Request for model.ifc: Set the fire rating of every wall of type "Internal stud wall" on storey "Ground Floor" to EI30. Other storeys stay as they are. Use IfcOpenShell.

First a look at what the model holds.

```python
import ifcopenshell
import ifcopenshell.util.element

model = ifcopenshell.open("model.ifc")
print(model.schema)
storey = next(s for s in model.by_type("IfcBuildingStorey") if s.Name == "Ground Floor")
walls = [e for e in ifcopenshell.util.element.get_decomposition(storey) if e.is_a("IfcWall")]
seen = {}
for e in walls:
    element_type = ifcopenshell.util.element.get_type(e)
    key = (element_type.Name if element_type != e and element_type else None, ifcopenshell.util.element.get_pset(e, "Pset_WallCommon", "FireRating"))
    seen[key] = seen.get(key, 0) + 1
for (name, value), count in sorted(seen.items(), key=str):
    print(count, "x", name, "|", value)
```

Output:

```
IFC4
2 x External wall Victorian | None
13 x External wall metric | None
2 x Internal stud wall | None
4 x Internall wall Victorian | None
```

```python
import ifcopenshell
import ifcopenshell.api.pset
import ifcopenshell.util.element

model = ifcopenshell.open("model.ifc")

storey = next(s for s in model.by_type("IfcBuildingStorey") if s.Name == "Ground Floor")
walls = [e for e in ifcopenshell.util.element.get_decomposition(storey) if e.is_a("IfcWall")]

count = 0
for e in walls:
    element_type = ifcopenshell.util.element.get_type(e)
    if element_type in (None, e) or element_type.Name != "Internal stud wall":
        continue
    # add_pset returns the element's existing set when there is one.
    pset = ifcopenshell.api.pset.add_pset(model, product=e, name="Pset_WallCommon")
    ifcopenshell.api.pset.edit_pset(model, pset=pset, properties={"FireRating": "EI30"})
    count += 1

print(count, "walls updated")

model.write("model_rev.ifc")
```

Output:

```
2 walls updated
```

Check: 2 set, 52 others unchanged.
